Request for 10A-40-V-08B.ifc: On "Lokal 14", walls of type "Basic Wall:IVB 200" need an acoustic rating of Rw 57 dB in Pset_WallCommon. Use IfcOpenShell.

First a look at what the model holds.

```python
import ifcopenshell
import ifcopenshell.util.element

model = ifcopenshell.open("10A-40-V-08B.ifc")
print(model.schema)
storey = next(s for s in model.by_type("IfcBuildingStorey") if s.Name == "Lokal 14")
walls = [e for e in ifcopenshell.util.element.get_decomposition(storey) if e.is_a("IfcWall")]
seen = {}
for e in walls:
    element_type = ifcopenshell.util.element.get_type(e)
    key = (element_type.Name if element_type != e and element_type else None, ifcopenshell.util.element.get_pset(e, "Pset_WallCommon", "AcousticRating"))
    seen[key] = seen.get(key, 0) + 1
for (name, value), count in sorted(seen.items(), key=str):
    print(count, "x", name, "|", value)
```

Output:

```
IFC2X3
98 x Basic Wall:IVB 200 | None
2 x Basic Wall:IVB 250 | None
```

```python
import ifcopenshell
import ifcopenshell.api.pset
import ifcopenshell.util.element

model = ifcopenshell.open("10A-40-V-08B.ifc")

storey = next(s for s in model.by_type("IfcBuildingStorey") if s.Name == "Lokal 14")
walls = [e for e in ifcopenshell.util.element.get_decomposition(storey) if e.is_a("IfcWall")]

count = 0
for e in walls:
    element_type = ifcopenshell.util.element.get_type(e)
    if element_type in (None, e) or element_type.Name != "Basic Wall:IVB 200":
        continue
    found = ifcopenshell.util.element.get_pset(e, "Pset_WallCommon", should_inherit=False)
    if found:
        pset = model.by_id(found["id"])
        if len(ifcopenshell.util.element.get_elements_by_pset(pset)) > 1:
            pset = ifcopenshell.api.pset.unshare_pset(model, products=[e], pset=pset)[0]
    else:
        pset = ifcopenshell.api.pset.add_pset(model, product=e, name="Pset_WallCommon")
    ifcopenshell.api.pset.edit_pset(model, pset=pset, properties={"AcousticRating": "Rw 57 dB"})
    count += 1

print(count, "walls updated")

model.write("10A-40-V-08B-out.ifc")
```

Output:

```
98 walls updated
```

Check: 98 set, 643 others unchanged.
